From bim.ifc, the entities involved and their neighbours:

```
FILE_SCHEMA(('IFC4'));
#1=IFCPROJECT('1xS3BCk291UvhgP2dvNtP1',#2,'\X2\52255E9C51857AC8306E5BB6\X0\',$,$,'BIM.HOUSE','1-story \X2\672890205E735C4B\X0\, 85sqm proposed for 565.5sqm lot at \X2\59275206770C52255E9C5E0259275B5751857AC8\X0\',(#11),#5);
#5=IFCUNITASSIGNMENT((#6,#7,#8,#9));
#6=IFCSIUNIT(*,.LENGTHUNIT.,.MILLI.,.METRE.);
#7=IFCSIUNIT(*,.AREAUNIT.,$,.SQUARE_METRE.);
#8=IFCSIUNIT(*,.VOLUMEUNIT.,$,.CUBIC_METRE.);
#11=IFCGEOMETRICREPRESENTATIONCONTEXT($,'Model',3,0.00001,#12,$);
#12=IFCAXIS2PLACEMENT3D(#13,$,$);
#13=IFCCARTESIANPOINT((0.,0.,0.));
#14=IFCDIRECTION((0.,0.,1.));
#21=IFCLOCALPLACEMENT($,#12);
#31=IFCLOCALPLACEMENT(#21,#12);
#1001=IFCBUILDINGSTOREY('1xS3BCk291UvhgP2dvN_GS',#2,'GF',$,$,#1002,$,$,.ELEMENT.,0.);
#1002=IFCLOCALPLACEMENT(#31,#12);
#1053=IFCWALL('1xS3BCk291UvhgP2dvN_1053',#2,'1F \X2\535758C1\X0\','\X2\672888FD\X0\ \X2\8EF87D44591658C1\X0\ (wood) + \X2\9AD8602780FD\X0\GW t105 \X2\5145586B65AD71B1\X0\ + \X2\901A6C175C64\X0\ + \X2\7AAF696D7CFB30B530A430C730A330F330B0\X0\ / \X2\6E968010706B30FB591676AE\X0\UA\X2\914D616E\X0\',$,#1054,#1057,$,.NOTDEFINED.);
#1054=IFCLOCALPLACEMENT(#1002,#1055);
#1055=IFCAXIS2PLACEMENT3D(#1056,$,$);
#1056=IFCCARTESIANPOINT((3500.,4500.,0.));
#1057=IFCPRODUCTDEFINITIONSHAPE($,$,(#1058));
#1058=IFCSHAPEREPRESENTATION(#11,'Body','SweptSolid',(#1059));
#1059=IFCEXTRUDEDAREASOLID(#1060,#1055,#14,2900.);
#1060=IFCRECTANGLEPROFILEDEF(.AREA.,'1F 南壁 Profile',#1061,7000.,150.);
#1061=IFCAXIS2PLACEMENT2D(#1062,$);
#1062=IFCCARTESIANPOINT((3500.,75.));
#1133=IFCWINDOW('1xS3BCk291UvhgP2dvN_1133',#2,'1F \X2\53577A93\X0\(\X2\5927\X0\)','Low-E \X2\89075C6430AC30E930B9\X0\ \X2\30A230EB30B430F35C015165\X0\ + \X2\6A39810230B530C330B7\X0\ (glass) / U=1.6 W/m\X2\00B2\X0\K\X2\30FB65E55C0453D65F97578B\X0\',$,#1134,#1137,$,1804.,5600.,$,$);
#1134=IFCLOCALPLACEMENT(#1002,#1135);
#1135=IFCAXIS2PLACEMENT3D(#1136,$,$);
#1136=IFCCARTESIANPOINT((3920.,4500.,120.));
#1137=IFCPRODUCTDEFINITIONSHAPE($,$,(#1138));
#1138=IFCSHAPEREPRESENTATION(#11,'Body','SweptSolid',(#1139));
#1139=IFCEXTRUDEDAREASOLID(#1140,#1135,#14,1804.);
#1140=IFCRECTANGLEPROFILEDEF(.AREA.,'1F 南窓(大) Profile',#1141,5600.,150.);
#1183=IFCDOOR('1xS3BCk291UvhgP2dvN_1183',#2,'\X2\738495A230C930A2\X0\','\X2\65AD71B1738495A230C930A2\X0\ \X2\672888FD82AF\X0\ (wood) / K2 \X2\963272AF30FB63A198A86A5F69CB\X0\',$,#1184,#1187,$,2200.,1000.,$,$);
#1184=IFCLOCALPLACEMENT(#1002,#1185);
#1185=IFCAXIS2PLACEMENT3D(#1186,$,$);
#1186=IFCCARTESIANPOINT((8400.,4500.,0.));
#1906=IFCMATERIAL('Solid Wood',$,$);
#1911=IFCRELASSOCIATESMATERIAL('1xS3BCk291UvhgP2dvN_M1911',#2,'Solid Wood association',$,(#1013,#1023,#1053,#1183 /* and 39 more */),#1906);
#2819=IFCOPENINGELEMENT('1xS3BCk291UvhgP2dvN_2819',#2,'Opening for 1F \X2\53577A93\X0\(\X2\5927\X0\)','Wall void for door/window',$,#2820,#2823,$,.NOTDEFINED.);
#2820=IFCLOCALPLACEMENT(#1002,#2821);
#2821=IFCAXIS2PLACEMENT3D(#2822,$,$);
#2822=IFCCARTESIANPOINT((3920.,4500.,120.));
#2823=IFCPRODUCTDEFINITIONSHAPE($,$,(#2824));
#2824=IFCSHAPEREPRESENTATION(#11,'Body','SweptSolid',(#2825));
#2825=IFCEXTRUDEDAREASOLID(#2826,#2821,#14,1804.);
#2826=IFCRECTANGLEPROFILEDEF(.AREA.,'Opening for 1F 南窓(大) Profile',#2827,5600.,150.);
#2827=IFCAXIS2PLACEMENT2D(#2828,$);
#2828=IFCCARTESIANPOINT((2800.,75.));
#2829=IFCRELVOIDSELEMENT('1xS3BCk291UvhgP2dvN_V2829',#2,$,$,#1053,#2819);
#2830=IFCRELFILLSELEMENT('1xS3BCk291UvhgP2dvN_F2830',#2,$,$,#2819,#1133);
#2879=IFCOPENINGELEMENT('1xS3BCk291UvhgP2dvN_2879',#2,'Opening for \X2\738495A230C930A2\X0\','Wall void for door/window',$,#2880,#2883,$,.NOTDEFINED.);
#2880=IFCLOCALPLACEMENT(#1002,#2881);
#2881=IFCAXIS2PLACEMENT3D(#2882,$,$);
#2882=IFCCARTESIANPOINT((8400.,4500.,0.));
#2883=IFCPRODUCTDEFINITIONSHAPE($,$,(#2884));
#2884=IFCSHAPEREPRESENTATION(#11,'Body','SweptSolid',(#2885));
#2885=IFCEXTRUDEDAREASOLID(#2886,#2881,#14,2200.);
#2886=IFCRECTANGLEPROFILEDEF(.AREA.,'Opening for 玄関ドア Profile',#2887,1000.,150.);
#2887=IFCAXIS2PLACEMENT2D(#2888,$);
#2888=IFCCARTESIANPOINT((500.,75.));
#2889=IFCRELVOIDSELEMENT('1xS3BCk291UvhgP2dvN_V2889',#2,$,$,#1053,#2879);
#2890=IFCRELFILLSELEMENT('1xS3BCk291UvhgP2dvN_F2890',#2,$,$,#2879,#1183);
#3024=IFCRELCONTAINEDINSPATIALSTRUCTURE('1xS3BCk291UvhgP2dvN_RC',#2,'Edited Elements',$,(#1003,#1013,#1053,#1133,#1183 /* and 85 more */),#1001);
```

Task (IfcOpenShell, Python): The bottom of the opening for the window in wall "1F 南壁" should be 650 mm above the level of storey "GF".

```python
import numpy as np
import ifcopenshell
import ifcopenshell.api.geometry
import ifcopenshell.geom
import ifcopenshell.util.element
import ifcopenshell.util.placement
import ifcopenshell.util.shape
import ifcopenshell.util.unit

model = ifcopenshell.open("bim.ifc")
unit_scale = ifcopenshell.util.unit.calculate_unit_scale(model)

window = model.by_id(1133)
opening = window.FillsVoids[0].RelatingOpeningElement
storey = ifcopenshell.util.element.get_container(window, ifc_class="IfcBuildingStorey")
level = ifcopenshell.util.placement.get_local_placement(storey.ObjectPlacement)[2, 3]

# The opening's origin need not be at the sill, so measure its lowest point.
shape = ifcopenshell.geom.create_shape(ifcopenshell.geom.settings(), opening)
bottom = ifcopenshell.util.shape.get_shape_bottom_elevation(shape, shape.geometry) / unit_scale
dz = level + 0.65 / unit_scale - bottom

shift = np.array([0.0, 0.0, dz])
# The window is not placed relative to its opening, so move both.
for product in (opening, window):
    matrix = ifcopenshell.util.placement.get_local_placement(product.ObjectPlacement)
    matrix[:3, 3] += shift
    ifcopenshell.api.geometry.edit_object_placement(model, product=product, matrix=matrix, is_si=False)

print(f"moved by {dz * unit_scale:+.3f} m")

model.write("bim_v2.ifc")
```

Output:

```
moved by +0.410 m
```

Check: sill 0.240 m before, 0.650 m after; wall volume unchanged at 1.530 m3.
